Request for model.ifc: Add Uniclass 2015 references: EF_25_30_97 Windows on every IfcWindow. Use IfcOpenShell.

First a look at what the model holds.

```python
import ifcopenshell

model = ifcopenshell.open("model.ifc")
print(model.schema)
print("classifications:", [c.Name for c in model.by_type("IfcClassification")])
for ifc_class in ("IfcDoor", "IfcRoof", "IfcStair", "IfcWall", "IfcWindow"):
    print(ifc_class, len(model.by_type(ifc_class)))
```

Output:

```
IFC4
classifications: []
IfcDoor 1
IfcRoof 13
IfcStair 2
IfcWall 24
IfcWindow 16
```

```python
import ifcopenshell
import ifcopenshell.api.classification

model = ifcopenshell.open("model.ifc")

system = ifcopenshell.api.classification.add_classification(model, classification="Uniclass 2015")

codes = {
    "IfcWindow": ("EF_25_30_97", "Windows"),
}
for ifc_class, (code, name) in codes.items():
    products = model.by_type(ifc_class)
    ifcopenshell.api.classification.add_reference(
        model, products=products, classification=system, identification=code, name=name
    )
    print(code, len(products))

model.write("model_updated.ifc")
```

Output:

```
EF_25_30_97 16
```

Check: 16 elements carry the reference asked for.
